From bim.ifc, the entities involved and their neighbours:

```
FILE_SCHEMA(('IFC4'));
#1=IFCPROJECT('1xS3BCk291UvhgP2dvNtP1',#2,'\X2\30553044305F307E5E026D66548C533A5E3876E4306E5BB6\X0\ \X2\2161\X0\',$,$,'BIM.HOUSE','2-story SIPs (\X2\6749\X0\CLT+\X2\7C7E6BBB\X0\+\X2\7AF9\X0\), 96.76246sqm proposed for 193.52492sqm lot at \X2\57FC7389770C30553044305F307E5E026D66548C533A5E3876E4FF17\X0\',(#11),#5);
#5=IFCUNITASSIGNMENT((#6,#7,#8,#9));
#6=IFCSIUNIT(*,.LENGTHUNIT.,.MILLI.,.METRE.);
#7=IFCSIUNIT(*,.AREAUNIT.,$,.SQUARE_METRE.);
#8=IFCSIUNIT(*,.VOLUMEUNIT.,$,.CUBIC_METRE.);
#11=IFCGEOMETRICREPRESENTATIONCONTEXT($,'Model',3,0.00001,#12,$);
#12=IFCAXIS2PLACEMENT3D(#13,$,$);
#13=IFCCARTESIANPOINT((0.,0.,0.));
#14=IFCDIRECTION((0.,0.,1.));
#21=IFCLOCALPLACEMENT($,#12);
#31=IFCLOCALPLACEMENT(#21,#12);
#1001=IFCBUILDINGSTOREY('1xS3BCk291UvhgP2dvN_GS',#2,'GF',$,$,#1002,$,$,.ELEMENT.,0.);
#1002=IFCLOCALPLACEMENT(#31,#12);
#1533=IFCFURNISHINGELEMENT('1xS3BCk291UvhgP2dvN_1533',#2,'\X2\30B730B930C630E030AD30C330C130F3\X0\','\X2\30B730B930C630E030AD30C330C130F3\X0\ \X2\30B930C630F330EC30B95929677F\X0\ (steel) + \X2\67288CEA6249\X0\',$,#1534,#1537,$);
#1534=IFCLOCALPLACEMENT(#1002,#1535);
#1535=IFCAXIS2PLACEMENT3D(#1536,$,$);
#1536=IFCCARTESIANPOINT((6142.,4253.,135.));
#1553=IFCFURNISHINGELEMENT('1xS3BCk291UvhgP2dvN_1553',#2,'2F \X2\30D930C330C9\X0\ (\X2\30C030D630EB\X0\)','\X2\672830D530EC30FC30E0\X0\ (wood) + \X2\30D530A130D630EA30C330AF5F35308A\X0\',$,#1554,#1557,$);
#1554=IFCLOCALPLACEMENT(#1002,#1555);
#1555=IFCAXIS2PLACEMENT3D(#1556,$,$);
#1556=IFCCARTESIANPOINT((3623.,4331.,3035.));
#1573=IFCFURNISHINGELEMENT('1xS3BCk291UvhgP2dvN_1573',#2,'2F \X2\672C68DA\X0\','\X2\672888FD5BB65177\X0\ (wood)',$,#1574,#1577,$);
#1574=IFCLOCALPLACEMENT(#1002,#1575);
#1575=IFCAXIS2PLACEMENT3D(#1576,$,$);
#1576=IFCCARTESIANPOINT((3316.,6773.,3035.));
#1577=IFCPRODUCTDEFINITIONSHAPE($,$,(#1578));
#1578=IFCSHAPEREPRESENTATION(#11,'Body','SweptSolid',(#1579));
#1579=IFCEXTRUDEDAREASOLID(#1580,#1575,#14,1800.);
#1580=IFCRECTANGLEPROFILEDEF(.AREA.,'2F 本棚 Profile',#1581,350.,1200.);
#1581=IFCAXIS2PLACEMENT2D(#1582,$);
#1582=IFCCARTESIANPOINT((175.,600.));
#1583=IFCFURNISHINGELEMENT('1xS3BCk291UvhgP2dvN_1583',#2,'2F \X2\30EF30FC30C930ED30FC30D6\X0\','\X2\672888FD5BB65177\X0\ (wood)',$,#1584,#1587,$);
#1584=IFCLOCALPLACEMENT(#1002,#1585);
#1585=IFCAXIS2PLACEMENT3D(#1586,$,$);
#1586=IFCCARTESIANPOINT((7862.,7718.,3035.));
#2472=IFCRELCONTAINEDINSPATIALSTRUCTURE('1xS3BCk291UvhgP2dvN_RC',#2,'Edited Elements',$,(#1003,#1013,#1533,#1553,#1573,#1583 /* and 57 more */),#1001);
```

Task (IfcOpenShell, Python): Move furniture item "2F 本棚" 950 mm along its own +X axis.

```python
import ifcopenshell
import ifcopenshell.api.geometry
import ifcopenshell.util.placement
import ifcopenshell.util.unit

model = ifcopenshell.open("bim.ifc")
unit_scale = ifcopenshell.util.unit.calculate_unit_scale(model)

item = model.by_guid("1xS3BCk291UvhgP2dvN_1573")
matrix = ifcopenshell.util.placement.get_local_placement(item.ObjectPlacement)
matrix[:3, 3] += matrix[:3, 0] * 0.95 / unit_scale
ifcopenshell.api.geometry.edit_object_placement(model, product=item, matrix=matrix, is_si=False)

print(ifcopenshell.util.placement.get_local_placement(item.ObjectPlacement).round(3) + 0.0)

model.write("bim_rev.ifc")
```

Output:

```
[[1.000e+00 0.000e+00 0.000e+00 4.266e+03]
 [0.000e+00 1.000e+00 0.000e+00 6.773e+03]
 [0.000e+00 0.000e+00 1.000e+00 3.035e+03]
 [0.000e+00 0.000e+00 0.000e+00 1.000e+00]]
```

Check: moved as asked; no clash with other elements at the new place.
